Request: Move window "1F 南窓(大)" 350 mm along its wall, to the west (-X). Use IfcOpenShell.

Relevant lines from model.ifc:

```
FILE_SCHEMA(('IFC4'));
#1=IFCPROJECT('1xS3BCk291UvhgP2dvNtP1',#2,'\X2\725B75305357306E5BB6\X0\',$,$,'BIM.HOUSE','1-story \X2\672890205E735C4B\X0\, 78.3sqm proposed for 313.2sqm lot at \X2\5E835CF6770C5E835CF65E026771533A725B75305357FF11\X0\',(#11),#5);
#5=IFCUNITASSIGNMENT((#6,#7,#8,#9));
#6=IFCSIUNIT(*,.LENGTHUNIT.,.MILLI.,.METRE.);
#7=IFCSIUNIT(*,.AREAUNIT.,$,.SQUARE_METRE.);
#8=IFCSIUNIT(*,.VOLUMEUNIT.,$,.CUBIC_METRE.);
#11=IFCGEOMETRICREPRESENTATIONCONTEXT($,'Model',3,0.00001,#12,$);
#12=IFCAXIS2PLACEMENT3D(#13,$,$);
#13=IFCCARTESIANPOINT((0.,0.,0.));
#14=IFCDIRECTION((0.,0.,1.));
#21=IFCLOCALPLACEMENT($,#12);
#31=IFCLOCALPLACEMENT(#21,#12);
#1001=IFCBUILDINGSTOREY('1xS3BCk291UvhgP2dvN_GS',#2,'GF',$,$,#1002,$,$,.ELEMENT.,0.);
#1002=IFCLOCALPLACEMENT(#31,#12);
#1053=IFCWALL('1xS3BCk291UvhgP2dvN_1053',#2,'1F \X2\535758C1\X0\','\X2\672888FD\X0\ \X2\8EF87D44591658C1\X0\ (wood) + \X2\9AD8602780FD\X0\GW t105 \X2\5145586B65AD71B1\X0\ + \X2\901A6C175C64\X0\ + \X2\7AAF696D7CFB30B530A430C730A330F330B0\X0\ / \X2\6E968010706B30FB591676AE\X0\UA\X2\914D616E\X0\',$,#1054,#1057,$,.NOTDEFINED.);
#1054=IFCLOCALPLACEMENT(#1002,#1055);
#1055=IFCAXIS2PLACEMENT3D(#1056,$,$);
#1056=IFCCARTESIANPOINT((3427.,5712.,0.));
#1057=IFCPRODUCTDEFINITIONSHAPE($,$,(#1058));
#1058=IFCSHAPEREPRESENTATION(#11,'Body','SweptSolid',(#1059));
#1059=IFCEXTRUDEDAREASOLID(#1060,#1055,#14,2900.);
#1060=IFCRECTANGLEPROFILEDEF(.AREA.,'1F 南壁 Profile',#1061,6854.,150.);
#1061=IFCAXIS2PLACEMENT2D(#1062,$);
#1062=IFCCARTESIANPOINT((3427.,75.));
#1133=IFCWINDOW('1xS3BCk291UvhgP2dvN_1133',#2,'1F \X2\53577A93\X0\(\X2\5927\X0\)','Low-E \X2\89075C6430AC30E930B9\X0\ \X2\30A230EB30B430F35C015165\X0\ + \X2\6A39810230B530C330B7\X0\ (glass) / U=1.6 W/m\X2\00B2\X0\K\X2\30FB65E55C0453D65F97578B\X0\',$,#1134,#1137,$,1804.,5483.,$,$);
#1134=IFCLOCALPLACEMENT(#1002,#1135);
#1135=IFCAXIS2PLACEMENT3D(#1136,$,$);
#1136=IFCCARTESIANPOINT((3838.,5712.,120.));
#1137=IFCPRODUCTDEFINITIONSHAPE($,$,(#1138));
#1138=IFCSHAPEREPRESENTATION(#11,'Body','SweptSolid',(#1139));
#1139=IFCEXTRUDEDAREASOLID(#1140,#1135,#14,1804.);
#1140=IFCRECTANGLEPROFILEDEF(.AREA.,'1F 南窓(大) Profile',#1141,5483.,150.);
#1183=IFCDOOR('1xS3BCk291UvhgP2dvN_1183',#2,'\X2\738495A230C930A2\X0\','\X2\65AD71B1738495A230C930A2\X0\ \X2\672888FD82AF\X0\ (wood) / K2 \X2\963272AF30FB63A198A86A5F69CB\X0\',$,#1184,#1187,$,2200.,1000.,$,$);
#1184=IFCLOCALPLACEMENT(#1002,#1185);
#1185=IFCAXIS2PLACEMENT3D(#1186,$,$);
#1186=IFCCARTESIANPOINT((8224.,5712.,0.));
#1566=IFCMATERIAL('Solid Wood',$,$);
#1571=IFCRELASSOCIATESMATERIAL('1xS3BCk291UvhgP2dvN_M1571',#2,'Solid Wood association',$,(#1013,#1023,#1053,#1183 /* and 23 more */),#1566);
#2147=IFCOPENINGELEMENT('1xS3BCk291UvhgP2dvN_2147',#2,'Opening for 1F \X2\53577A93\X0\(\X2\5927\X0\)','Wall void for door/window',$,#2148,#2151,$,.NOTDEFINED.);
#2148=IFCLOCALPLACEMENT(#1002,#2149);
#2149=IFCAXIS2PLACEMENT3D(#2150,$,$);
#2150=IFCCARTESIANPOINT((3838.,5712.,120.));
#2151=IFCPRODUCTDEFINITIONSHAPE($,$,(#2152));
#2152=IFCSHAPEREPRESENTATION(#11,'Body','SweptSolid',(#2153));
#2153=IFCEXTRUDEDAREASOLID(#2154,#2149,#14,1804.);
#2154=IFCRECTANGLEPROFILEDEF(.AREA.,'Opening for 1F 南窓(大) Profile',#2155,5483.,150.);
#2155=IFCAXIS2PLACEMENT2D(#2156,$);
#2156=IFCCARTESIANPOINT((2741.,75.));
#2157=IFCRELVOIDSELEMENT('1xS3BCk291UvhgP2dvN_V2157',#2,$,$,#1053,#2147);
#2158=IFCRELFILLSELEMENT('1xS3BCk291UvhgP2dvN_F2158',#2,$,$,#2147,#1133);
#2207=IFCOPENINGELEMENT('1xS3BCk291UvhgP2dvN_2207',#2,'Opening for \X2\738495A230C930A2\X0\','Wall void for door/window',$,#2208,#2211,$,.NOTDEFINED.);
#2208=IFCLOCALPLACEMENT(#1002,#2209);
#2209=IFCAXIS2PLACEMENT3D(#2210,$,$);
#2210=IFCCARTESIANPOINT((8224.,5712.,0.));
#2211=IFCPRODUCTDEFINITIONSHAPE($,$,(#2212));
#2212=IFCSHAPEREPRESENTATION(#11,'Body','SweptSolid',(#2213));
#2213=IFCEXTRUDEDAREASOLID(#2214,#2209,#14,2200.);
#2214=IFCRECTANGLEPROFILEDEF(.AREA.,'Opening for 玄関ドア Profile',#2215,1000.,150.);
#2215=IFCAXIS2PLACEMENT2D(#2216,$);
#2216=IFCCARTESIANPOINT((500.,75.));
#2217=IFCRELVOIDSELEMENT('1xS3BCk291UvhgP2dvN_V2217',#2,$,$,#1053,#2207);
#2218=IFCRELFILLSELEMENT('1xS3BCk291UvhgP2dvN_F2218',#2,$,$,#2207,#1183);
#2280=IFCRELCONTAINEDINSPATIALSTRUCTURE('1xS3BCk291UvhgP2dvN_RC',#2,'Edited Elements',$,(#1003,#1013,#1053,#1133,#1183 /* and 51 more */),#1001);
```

```python
import ifcopenshell
import ifcopenshell.api.geometry
import ifcopenshell.util.placement

model = ifcopenshell.open("model.ifc")

window = model.by_guid("1xS3BCk291UvhgP2dvN_1133")
opening = window.FillsVoids[0].RelatingOpeningElement
wall = opening.VoidsElements[0].RelatingBuildingElement

wall_matrix = ifcopenshell.util.placement.get_local_placement(wall.ObjectPlacement)
shift = wall_matrix[:3, 0] * -350.0
before = ifcopenshell.util.placement.get_local_placement(window.ObjectPlacement)[:3, 3].copy()

# The window is not placed relative to its opening, so move both.
for product in (opening, window):
    matrix = ifcopenshell.util.placement.get_local_placement(product.ObjectPlacement)
    matrix[:3, 3] += shift
    ifcopenshell.api.geometry.edit_object_placement(model, product=product, matrix=matrix, is_si=False)

after = ifcopenshell.util.placement.get_local_placement(window.ObjectPlacement)[:3, 3]
print("window moved by", (after - before).round(3) + 0.0)

model.write("model_rev.ifc")
```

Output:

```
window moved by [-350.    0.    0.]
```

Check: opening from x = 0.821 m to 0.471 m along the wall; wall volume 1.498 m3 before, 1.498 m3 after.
